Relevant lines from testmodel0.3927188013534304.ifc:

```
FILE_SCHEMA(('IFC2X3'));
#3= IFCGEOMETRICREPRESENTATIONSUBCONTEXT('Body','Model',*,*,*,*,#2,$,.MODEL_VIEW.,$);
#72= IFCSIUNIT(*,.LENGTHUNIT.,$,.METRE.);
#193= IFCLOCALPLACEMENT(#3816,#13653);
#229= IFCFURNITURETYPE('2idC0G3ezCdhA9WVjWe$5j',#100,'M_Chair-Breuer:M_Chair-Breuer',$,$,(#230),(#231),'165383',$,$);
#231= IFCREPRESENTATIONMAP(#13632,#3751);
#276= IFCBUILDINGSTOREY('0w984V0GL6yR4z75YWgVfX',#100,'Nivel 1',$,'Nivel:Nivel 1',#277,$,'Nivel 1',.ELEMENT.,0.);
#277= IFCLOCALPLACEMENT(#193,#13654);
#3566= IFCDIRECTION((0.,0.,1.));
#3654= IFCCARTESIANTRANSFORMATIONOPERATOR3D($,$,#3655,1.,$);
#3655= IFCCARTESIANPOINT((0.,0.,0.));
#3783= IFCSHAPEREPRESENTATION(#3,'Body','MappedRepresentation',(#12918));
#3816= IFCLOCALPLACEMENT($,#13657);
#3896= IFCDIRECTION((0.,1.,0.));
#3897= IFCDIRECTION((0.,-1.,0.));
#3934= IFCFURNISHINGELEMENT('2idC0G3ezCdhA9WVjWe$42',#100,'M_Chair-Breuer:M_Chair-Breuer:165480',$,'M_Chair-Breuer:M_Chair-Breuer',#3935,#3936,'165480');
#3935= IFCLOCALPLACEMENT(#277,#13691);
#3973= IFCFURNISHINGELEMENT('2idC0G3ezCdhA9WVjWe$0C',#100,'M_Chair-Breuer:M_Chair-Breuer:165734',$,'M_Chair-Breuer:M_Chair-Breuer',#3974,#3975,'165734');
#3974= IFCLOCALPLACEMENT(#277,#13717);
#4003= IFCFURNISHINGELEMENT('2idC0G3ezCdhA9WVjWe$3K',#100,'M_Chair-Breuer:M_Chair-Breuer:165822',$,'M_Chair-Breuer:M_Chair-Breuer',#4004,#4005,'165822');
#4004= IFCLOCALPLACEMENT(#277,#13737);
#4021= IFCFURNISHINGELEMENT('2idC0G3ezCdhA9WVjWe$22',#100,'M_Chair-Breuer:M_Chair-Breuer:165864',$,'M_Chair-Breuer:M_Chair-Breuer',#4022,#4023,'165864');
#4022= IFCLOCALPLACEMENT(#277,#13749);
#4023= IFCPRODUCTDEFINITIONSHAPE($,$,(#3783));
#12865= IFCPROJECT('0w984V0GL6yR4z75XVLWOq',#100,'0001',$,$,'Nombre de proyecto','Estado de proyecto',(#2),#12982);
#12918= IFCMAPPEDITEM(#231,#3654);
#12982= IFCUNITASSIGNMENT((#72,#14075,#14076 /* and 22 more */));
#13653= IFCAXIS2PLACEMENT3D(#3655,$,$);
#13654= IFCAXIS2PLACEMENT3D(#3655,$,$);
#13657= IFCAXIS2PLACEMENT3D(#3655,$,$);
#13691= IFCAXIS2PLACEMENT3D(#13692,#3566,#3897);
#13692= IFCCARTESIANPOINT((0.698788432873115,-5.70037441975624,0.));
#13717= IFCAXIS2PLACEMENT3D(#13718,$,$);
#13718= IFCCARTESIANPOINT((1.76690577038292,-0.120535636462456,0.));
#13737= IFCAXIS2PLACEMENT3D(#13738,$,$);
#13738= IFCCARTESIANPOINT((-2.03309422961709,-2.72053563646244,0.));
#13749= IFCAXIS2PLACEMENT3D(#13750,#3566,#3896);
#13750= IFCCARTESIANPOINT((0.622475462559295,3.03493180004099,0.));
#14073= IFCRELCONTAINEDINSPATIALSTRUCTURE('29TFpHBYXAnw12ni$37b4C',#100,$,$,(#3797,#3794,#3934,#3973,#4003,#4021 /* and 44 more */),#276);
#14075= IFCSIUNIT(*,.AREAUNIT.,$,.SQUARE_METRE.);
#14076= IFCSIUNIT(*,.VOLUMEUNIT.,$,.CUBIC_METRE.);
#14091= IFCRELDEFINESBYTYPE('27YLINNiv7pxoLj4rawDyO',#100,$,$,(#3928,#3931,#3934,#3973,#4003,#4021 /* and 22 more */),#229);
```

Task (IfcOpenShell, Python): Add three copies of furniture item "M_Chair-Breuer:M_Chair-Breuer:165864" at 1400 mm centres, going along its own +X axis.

```python
import ifcopenshell
import ifcopenshell.api.geometry
import ifcopenshell.api.root
import ifcopenshell.util.element
import ifcopenshell.util.placement
import ifcopenshell.util.unit

model = ifcopenshell.open("testmodel0.3927188013534304.ifc")
unit_scale = ifcopenshell.util.unit.calculate_unit_scale(model)


def reuse_history(source, copy):
    """copy_class also copies each property set's owner history, people and application; keep the originals."""
    for rel in copy.IsDefinedBy:
        if rel.is_a("IfcRelDefinesByProperties") and (history := rel.RelatingPropertyDefinition.OwnerHistory):
            rel.RelatingPropertyDefinition.OwnerHistory = source.OwnerHistory
            ifcopenshell.util.element.remove_deep2(model, history)


source = model.by_guid("2idC0G3ezCdhA9WVjWe$22")
base = ifcopenshell.util.placement.get_local_placement(source.ObjectPlacement)
step = base[:3, 0] * 1.4 / unit_scale

for i in range(1, 4):
    copy = ifcopenshell.api.root.copy_class(model, product=source)
    copy.Representation = ifcopenshell.util.element.copy_deep(
        model, source.Representation, exclude=["IfcGeometricRepresentationContext", "IfcRepresentationMap"]
    )
    copy.Name = "M_Chair-Breuer:M_Chair-Breuer"
    copy.Tag = None
    reuse_history(source, copy)
    matrix = base.copy()
    matrix[:3, 3] += i * step
    print("added at", matrix[:3, 3].round(3) + 0.0)
    ifcopenshell.api.geometry.edit_object_placement(model, product=copy, matrix=matrix, is_si=False)

model.write("testmodel0.3927188013534304-out.ifc")
```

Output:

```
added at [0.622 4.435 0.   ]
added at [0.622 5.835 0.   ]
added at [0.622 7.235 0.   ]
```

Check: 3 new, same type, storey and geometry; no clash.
